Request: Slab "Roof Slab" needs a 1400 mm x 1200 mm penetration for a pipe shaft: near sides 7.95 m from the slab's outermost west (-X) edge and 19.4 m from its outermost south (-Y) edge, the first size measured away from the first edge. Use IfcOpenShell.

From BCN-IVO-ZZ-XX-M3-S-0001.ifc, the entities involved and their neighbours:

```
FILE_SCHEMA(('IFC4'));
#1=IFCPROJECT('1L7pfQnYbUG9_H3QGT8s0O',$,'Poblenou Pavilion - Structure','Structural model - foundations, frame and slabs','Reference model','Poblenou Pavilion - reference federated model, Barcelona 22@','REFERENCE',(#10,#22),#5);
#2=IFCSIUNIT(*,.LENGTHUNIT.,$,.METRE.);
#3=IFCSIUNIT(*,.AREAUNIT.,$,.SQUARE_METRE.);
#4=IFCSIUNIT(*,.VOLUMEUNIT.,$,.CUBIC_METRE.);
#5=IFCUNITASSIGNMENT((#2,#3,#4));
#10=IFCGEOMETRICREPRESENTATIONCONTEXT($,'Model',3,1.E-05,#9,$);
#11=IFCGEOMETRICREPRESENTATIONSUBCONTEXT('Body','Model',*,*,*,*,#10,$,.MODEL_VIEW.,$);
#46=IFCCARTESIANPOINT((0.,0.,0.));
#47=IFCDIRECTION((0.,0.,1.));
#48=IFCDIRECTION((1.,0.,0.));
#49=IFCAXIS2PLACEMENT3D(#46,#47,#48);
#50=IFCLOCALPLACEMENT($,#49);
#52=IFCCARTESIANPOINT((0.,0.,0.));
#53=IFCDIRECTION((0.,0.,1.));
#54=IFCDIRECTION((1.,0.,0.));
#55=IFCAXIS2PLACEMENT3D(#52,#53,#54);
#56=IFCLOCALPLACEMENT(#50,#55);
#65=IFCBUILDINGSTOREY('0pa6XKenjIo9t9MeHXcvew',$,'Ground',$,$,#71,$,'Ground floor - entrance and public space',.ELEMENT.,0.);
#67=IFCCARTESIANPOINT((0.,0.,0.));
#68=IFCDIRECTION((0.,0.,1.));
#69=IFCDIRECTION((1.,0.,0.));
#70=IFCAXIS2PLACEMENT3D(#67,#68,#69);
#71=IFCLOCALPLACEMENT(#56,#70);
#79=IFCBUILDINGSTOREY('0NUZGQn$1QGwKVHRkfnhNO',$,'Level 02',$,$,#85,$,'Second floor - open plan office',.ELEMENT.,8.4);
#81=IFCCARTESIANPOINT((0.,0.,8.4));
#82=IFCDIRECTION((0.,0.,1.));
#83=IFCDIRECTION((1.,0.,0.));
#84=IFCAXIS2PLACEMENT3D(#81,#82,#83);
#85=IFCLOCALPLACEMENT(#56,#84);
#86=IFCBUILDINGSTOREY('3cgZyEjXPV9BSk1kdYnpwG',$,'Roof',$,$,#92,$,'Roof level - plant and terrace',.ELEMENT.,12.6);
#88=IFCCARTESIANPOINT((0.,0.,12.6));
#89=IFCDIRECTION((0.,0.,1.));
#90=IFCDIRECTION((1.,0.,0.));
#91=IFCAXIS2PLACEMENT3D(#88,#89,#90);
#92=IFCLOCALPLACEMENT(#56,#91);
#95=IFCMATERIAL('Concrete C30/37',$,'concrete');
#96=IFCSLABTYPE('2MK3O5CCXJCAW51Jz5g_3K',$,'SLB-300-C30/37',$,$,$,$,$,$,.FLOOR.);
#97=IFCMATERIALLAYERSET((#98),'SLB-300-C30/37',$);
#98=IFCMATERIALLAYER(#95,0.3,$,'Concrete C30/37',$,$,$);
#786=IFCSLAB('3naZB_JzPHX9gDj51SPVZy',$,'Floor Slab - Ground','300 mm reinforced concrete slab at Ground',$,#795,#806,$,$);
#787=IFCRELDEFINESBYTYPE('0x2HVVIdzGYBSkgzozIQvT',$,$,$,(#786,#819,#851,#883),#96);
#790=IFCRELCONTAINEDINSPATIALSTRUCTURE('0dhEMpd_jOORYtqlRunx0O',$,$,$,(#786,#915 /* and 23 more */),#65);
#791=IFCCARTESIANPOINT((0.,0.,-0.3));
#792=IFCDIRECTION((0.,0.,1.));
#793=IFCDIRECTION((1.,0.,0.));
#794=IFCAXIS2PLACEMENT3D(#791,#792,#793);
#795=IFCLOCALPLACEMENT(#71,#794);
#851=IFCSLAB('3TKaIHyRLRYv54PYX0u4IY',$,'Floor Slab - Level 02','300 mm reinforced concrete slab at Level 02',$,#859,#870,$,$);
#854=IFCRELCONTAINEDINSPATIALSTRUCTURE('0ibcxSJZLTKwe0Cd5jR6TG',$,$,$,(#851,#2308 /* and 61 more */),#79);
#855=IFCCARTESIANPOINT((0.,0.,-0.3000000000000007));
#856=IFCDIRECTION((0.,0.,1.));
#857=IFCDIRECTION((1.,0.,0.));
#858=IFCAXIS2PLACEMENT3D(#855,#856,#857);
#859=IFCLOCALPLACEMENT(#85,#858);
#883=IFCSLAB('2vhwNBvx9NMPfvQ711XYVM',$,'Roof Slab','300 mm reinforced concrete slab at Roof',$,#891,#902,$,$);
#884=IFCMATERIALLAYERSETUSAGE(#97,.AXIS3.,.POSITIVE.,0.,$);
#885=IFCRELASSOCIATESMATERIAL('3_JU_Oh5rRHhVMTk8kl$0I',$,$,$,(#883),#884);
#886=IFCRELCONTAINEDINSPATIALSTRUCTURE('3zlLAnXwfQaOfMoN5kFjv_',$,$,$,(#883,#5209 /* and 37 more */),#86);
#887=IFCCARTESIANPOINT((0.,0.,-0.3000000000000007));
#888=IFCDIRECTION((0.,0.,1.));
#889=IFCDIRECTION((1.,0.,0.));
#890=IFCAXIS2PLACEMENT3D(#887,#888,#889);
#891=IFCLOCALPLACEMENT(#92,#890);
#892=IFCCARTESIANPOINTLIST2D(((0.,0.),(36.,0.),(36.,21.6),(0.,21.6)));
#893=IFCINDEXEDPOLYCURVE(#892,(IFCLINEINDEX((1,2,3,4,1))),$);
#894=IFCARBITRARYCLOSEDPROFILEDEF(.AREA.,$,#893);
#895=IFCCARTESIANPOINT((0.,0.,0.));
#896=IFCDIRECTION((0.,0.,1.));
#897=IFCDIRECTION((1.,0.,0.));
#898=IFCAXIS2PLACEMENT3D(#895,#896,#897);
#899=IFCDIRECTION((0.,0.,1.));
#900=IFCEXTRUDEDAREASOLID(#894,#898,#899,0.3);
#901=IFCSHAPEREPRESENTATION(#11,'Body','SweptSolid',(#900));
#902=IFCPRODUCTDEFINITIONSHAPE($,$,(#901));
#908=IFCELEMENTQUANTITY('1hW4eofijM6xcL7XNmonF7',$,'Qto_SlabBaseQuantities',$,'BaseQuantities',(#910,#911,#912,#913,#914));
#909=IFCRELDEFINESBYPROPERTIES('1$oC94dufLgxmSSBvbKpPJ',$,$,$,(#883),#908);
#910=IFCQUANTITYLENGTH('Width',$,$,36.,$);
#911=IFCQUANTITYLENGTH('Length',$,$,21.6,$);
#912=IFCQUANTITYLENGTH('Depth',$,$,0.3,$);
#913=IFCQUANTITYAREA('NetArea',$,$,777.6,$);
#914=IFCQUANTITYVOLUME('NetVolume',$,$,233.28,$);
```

```python
import numpy as np
import ifcopenshell
import ifcopenshell.api.feature
import ifcopenshell.api.geometry
import ifcopenshell.api.pset
import ifcopenshell.api.root
import ifcopenshell.geom
import ifcopenshell.util.element
import ifcopenshell.util.placement
import ifcopenshell.util.representation
import ifcopenshell.util.shape
import ifcopenshell.util.unit

model = ifcopenshell.open("BCN-IVO-ZZ-XX-M3-S-0001.ifc")
unit_scale = ifcopenshell.util.unit.calculate_unit_scale(model)
area_scale = ifcopenshell.util.unit.calculate_unit_scale(model, "AREAUNIT")
volume_scale = ifcopenshell.util.unit.calculate_unit_scale(model, "VOLUMEUNIT")
settings = ifcopenshell.geom.settings()


def volume(element):
    """Net volume in cubic metres, openings subtracted."""
    shape = ifcopenshell.geom.create_shape(settings, element)
    return ifcopenshell.util.shape.get_volume(shape.geometry)


slab = model.by_guid("2vhwNBvx9NMPfvQ711XYVM")
before = volume(slab)

# Extent in the slab's own axes, in metres. The edges named are its -X and -Y sides.
slab_shape = ifcopenshell.geom.create_shape(settings, slab)
vertices = ifcopenshell.util.shape.get_vertices(slab_shape.geometry)
x_min, y_min, bottom = vertices.min(axis=0)
top = vertices[:, 2].max()

opening = ifcopenshell.api.root.create_entity(model, ifc_class="IfcOpeningElement", name="Pipe shaft opening", predefined_type="OPENING")
context = ifcopenshell.util.representation.get_context(model, "Model", "Body", "MODEL_VIEW")
width, depth = 1.4, 1.2
outline = [(0.0, 0.0), (width, 0.0), (width, depth), (0.0, depth), (0.0, 0.0)]
# Overshoot both faces by 50 mm so the cut is clean.
shape = ifcopenshell.api.geometry.add_slab_representation(
    model, context=context, depth=top - bottom + 0.1, polyline=outline
)
ifcopenshell.api.geometry.assign_representation(model, product=opening, representation=shape)

matrix = ifcopenshell.util.placement.get_local_placement(slab.ObjectPlacement)
matrix[:, 3] = matrix @ np.append(np.array([x_min + 7.95, y_min + 19.4, bottom - 0.05]) / unit_scale, 1.0)
ifcopenshell.api.geometry.edit_object_placement(model, product=opening, matrix=matrix, is_si=False)
ifcopenshell.api.feature.add_feature(model, feature=opening, element=slab)

after = volume(slab)

# Update the slab's stored quantities.
qto = model.by_id(ifcopenshell.util.element.get_pset(slab, "Qto_SlabBaseQuantities", should_inherit=False)["id"])
ifcopenshell.api.pset.edit_qto(model, qto=qto, properties={
    "NetArea": after / (top - bottom) / area_scale,
    "NetVolume": after / volume_scale,
})

print(f"slab volume {before:.3f} -> {after:.3f} m3")

model.write("BCN-IVO-ZZ-XX-M3-S-0001_edited.ifc")
```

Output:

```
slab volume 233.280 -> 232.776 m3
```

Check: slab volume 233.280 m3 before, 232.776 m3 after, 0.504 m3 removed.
